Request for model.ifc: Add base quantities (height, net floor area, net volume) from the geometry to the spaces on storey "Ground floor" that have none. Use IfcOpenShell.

First a look at what the model holds.

```python
import ifcopenshell
import ifcopenshell.util.element
import ifcopenshell.util.unit

model = ifcopenshell.open("model.ifc")
print(model.schema)
for unit_type in ("LENGTHUNIT", "AREAUNIT", "VOLUMEUNIT"):
    print(unit_type, ifcopenshell.util.unit.calculate_unit_scale(model, unit_type))
storey = next(s for s in model.by_type("IfcBuildingStorey") if s.Name == "Ground floor")
spaces = [e for e in ifcopenshell.util.element.get_decomposition(storey) if e.is_a("IfcSpace")]
for e in sorted(spaces, key=lambda e: e.id()):
    print(e.id(), e.is_a(), e.Name, list(ifcopenshell.util.element.get_psets(e, qtos_only=True)), sep=" | ")
```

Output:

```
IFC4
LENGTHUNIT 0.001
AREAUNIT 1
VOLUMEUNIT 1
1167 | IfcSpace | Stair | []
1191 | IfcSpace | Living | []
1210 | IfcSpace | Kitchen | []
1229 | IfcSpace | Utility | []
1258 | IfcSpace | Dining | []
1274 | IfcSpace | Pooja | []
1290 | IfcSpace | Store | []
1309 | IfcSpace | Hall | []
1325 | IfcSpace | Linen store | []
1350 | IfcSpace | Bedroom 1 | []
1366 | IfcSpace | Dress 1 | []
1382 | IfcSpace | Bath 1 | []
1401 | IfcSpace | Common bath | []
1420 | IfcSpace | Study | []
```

```python
import ifcopenshell
import ifcopenshell.api.pset
import ifcopenshell.geom
import ifcopenshell.util.element
import ifcopenshell.util.shape
import ifcopenshell.util.unit

model = ifcopenshell.open("model.ifc")
unit_scale = ifcopenshell.util.unit.calculate_unit_scale(model)
area_scale = ifcopenshell.util.unit.calculate_unit_scale(model, "AREAUNIT")
volume_scale = ifcopenshell.util.unit.calculate_unit_scale(model, "VOLUMEUNIT")
settings = ifcopenshell.geom.settings()

storey = next(s for s in model.by_type("IfcBuildingStorey") if s.Name == "Ground floor")
spaces = [e for e in ifcopenshell.util.element.get_decomposition(storey) if e.is_a("IfcSpace")]

for e in sorted(spaces, key=lambda e: e.id()):
    if ifcopenshell.util.element.get_psets(e, qtos_only=True, should_inherit=False):
        continue
    # Geometry comes back in metres, in the element's own axes.
    shape = ifcopenshell.geom.create_shape(settings, e)
    values = {
        "Height": ifcopenshell.util.shape.get_z(shape.geometry) / unit_scale,
        "NetFloorArea": ifcopenshell.util.shape.get_footprint_area(shape.geometry) / area_scale,
        "NetVolume": ifcopenshell.util.shape.get_volume(shape.geometry) / volume_scale,
    }
    qto = ifcopenshell.api.pset.add_qto(model, product=e, name="Qto_SpaceBaseQuantities")
    ifcopenshell.api.pset.edit_qto(model, qto=qto, properties=values)
    print(e.id(), {k: round(v, 3) for k, v in values.items()})

model.write("model_v2.ifc")
```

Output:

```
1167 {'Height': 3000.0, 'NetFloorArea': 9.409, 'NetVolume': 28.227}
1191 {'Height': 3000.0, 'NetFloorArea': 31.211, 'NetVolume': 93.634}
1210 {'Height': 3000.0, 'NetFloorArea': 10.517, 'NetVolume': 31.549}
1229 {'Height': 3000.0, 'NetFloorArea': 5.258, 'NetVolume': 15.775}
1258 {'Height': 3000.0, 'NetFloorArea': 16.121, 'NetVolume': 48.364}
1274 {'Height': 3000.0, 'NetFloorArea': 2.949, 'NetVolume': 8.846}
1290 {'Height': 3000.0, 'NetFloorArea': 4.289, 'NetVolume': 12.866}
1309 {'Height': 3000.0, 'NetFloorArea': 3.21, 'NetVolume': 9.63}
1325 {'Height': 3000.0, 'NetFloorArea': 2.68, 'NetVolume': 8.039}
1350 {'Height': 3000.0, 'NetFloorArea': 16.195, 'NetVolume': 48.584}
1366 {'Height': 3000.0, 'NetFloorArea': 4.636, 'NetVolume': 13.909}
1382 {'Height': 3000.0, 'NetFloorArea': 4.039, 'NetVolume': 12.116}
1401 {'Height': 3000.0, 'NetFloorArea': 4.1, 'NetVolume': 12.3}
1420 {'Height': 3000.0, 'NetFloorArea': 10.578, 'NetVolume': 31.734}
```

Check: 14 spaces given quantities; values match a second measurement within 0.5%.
